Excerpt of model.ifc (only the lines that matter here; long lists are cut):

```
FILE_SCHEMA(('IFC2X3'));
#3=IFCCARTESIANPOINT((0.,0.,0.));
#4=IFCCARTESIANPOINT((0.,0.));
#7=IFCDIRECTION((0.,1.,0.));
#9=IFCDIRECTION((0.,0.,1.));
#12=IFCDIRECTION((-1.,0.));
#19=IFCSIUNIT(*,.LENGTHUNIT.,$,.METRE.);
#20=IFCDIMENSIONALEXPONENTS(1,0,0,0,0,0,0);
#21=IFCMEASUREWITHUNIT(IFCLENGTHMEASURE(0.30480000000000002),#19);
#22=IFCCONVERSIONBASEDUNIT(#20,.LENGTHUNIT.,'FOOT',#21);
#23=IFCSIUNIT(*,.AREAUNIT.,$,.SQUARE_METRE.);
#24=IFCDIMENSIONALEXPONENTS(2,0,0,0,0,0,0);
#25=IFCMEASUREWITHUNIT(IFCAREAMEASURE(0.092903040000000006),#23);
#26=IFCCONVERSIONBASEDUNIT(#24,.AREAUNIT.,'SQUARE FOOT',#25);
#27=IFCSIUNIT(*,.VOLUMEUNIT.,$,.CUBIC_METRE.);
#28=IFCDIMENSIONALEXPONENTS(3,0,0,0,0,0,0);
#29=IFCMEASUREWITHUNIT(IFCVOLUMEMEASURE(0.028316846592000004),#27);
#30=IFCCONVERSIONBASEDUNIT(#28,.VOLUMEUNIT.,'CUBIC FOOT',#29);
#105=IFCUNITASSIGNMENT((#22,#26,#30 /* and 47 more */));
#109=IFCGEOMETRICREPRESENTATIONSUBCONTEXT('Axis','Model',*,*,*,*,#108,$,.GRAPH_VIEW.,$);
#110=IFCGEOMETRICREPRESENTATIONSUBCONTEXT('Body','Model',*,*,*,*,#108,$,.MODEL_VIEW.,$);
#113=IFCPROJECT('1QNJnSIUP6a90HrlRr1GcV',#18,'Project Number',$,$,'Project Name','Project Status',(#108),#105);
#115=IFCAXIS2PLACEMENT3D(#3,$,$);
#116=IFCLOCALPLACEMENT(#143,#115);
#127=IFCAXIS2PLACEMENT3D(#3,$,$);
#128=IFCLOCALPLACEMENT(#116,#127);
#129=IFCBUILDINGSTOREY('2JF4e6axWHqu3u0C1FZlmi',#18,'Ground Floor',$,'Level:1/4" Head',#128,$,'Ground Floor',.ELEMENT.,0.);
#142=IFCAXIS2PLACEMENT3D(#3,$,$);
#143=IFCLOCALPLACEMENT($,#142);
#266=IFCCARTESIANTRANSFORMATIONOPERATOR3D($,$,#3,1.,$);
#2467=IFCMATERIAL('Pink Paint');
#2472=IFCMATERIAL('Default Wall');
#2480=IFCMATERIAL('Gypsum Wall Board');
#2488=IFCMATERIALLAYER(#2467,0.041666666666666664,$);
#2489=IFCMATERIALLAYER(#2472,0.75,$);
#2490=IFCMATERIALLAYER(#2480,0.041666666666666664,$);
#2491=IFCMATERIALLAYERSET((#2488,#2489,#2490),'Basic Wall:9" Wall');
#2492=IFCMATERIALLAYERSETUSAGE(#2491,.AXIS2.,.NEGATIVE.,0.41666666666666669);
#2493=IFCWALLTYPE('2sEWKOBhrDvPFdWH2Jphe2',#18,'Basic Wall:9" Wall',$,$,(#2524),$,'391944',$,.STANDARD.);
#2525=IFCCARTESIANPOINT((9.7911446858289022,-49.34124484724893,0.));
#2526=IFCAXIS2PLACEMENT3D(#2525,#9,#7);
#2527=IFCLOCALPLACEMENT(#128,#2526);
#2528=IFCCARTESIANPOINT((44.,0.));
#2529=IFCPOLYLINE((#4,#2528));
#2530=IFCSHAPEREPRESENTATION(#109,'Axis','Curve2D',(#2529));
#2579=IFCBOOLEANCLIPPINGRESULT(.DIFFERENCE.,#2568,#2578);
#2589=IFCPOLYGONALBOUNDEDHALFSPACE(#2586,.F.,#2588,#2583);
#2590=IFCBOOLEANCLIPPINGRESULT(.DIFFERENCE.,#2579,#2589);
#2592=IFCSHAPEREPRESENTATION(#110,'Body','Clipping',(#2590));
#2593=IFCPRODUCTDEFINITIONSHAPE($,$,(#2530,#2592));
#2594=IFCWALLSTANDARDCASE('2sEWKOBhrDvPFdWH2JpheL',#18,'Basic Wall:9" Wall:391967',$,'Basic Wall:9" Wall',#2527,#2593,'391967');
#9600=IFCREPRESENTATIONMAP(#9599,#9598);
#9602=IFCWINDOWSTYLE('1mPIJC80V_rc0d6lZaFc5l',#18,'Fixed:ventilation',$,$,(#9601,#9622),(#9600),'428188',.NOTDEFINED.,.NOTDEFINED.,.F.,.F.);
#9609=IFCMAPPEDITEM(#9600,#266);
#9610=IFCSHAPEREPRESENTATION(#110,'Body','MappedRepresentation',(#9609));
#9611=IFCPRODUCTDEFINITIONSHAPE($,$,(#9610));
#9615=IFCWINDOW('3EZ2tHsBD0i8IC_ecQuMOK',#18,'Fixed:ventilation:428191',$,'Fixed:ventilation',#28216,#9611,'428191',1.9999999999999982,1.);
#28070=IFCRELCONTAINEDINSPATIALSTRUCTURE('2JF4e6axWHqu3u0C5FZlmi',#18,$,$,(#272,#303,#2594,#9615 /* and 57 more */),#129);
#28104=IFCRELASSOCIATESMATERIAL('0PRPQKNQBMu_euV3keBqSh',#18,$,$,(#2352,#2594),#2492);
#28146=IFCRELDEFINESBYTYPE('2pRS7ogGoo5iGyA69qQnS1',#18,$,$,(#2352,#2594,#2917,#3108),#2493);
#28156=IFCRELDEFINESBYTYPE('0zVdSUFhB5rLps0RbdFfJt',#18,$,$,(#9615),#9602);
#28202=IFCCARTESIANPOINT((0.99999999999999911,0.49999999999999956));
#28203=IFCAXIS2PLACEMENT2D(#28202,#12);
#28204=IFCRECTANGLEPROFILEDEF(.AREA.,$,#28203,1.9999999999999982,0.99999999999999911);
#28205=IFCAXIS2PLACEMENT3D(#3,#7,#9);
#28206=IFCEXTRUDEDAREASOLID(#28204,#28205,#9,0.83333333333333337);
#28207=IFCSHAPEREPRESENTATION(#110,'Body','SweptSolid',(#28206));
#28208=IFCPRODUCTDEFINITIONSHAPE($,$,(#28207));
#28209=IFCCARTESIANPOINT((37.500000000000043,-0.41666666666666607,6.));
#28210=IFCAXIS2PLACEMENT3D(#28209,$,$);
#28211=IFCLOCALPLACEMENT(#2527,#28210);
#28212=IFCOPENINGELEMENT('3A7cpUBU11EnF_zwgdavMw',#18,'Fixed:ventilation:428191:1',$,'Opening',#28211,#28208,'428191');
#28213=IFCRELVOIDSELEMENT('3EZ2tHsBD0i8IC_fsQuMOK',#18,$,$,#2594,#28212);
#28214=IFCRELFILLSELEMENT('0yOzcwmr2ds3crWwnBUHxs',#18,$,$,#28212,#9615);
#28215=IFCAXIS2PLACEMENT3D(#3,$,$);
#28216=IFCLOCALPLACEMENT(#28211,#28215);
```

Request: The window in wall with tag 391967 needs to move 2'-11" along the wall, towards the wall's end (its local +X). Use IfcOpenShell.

```python
import ifcopenshell
import ifcopenshell.api.geometry
import ifcopenshell.util.placement
import ifcopenshell.util.unit

model = ifcopenshell.open("model.ifc")
unit_scale = ifcopenshell.util.unit.calculate_unit_scale(model)

window = model.by_guid("3EZ2tHsBD0i8IC_ecQuMOK")
opening = window.FillsVoids[0].RelatingOpeningElement
wall = opening.VoidsElements[0].RelatingBuildingElement

wall_matrix = ifcopenshell.util.placement.get_local_placement(wall.ObjectPlacement)
shift = wall_matrix[:3, 0] * 35 * 0.0254 / unit_scale
before = ifcopenshell.util.placement.get_local_placement(window.ObjectPlacement)[:3, 3].copy()

# The window is placed relative to its opening, so it follows when the opening moves.
matrix = ifcopenshell.util.placement.get_local_placement(opening.ObjectPlacement)
matrix[:3, 3] += shift
ifcopenshell.api.geometry.edit_object_placement(
    model, product=opening, matrix=matrix, is_si=False, should_transform_children=True
)

after = ifcopenshell.util.placement.get_local_placement(window.ObjectPlacement)[:3, 3]
print("window moved by", (after - before).round(3) + 0.0)

model.write("model_v2.ifc")
```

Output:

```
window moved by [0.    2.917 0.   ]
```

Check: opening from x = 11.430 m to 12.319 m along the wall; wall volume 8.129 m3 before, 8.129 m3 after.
